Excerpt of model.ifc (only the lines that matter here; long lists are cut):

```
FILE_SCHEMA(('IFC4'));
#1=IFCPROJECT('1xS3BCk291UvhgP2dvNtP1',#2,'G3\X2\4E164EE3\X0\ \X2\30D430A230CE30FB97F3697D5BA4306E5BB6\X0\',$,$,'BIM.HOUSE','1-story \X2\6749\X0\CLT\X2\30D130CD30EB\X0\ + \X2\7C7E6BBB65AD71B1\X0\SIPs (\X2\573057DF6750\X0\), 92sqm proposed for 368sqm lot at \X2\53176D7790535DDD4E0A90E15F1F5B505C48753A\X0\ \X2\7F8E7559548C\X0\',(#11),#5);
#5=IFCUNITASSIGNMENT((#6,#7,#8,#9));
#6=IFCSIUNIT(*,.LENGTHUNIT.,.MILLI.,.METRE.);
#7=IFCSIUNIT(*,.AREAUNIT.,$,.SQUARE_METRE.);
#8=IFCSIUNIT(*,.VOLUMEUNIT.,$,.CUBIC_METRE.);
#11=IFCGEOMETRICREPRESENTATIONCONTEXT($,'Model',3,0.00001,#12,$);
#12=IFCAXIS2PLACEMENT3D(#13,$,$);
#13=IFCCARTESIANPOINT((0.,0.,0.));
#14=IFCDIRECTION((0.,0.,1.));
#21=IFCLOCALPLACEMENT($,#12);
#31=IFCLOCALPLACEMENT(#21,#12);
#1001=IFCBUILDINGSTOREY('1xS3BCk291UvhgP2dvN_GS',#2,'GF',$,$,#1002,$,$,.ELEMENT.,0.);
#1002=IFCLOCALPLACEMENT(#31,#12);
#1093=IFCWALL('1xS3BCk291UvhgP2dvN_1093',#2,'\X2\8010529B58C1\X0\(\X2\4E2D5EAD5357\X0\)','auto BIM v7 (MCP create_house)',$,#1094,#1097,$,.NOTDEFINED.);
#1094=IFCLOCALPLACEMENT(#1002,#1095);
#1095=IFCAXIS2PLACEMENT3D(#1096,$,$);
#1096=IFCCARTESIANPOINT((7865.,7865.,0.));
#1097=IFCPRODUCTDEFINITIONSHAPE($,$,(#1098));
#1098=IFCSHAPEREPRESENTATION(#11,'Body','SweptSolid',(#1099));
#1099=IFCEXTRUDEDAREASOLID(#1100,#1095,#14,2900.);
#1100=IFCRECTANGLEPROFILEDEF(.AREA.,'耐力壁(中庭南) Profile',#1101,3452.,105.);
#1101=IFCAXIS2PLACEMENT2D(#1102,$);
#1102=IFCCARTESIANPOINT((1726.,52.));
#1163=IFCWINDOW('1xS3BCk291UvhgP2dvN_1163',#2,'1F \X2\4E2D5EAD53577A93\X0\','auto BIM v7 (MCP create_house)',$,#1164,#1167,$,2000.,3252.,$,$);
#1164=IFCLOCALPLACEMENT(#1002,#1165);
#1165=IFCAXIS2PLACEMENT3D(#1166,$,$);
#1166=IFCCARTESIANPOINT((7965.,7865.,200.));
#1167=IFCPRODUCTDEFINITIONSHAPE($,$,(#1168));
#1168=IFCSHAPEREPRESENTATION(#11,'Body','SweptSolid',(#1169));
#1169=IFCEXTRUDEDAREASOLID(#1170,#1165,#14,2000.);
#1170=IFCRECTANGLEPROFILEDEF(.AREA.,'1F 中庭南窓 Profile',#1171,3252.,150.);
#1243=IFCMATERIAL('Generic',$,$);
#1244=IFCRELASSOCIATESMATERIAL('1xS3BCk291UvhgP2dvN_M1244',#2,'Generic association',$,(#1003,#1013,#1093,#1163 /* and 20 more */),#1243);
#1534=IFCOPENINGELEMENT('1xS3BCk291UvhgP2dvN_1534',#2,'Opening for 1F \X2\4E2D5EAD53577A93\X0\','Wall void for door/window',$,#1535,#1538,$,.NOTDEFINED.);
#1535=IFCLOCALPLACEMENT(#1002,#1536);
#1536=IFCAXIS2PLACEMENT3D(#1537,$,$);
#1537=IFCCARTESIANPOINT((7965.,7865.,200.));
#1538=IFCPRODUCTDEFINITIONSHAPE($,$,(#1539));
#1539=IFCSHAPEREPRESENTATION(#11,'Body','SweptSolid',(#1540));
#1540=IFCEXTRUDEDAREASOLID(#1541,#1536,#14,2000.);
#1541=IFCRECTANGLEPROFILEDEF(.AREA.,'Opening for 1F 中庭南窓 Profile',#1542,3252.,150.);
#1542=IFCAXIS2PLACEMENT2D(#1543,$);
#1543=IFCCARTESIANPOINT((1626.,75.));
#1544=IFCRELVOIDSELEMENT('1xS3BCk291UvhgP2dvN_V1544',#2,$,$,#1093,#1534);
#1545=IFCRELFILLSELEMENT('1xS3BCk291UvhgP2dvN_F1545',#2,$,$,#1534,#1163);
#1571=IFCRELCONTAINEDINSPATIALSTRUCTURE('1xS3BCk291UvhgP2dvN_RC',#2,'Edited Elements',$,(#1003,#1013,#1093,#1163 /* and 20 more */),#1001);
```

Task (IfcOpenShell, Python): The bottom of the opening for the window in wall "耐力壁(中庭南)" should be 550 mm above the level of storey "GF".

```python
import numpy as np
import ifcopenshell
import ifcopenshell.api.geometry
import ifcopenshell.geom
import ifcopenshell.util.element
import ifcopenshell.util.placement
import ifcopenshell.util.shape
import ifcopenshell.util.unit

model = ifcopenshell.open("model.ifc")
unit_scale = ifcopenshell.util.unit.calculate_unit_scale(model)

window = model.by_id(1163)
opening = window.FillsVoids[0].RelatingOpeningElement
storey = ifcopenshell.util.element.get_container(window, ifc_class="IfcBuildingStorey")
level = ifcopenshell.util.placement.get_local_placement(storey.ObjectPlacement)[2, 3]

# The opening's origin need not be at the sill, so measure its lowest point.
shape = ifcopenshell.geom.create_shape(ifcopenshell.geom.settings(), opening)
bottom = ifcopenshell.util.shape.get_shape_bottom_elevation(shape, shape.geometry) / unit_scale
dz = level + 0.55 / unit_scale - bottom

shift = np.array([0.0, 0.0, dz])
# The window is not placed relative to its opening, so move both.
for product in (opening, window):
    matrix = ifcopenshell.util.placement.get_local_placement(product.ObjectPlacement)
    matrix[:3, 3] += shift
    ifcopenshell.api.geometry.edit_object_placement(model, product=product, matrix=matrix, is_si=False)

print(f"moved by {dz * unit_scale:+.3f} m")

model.write("model_updated.ifc")
```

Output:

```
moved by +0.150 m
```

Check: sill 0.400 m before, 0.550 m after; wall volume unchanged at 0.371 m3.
